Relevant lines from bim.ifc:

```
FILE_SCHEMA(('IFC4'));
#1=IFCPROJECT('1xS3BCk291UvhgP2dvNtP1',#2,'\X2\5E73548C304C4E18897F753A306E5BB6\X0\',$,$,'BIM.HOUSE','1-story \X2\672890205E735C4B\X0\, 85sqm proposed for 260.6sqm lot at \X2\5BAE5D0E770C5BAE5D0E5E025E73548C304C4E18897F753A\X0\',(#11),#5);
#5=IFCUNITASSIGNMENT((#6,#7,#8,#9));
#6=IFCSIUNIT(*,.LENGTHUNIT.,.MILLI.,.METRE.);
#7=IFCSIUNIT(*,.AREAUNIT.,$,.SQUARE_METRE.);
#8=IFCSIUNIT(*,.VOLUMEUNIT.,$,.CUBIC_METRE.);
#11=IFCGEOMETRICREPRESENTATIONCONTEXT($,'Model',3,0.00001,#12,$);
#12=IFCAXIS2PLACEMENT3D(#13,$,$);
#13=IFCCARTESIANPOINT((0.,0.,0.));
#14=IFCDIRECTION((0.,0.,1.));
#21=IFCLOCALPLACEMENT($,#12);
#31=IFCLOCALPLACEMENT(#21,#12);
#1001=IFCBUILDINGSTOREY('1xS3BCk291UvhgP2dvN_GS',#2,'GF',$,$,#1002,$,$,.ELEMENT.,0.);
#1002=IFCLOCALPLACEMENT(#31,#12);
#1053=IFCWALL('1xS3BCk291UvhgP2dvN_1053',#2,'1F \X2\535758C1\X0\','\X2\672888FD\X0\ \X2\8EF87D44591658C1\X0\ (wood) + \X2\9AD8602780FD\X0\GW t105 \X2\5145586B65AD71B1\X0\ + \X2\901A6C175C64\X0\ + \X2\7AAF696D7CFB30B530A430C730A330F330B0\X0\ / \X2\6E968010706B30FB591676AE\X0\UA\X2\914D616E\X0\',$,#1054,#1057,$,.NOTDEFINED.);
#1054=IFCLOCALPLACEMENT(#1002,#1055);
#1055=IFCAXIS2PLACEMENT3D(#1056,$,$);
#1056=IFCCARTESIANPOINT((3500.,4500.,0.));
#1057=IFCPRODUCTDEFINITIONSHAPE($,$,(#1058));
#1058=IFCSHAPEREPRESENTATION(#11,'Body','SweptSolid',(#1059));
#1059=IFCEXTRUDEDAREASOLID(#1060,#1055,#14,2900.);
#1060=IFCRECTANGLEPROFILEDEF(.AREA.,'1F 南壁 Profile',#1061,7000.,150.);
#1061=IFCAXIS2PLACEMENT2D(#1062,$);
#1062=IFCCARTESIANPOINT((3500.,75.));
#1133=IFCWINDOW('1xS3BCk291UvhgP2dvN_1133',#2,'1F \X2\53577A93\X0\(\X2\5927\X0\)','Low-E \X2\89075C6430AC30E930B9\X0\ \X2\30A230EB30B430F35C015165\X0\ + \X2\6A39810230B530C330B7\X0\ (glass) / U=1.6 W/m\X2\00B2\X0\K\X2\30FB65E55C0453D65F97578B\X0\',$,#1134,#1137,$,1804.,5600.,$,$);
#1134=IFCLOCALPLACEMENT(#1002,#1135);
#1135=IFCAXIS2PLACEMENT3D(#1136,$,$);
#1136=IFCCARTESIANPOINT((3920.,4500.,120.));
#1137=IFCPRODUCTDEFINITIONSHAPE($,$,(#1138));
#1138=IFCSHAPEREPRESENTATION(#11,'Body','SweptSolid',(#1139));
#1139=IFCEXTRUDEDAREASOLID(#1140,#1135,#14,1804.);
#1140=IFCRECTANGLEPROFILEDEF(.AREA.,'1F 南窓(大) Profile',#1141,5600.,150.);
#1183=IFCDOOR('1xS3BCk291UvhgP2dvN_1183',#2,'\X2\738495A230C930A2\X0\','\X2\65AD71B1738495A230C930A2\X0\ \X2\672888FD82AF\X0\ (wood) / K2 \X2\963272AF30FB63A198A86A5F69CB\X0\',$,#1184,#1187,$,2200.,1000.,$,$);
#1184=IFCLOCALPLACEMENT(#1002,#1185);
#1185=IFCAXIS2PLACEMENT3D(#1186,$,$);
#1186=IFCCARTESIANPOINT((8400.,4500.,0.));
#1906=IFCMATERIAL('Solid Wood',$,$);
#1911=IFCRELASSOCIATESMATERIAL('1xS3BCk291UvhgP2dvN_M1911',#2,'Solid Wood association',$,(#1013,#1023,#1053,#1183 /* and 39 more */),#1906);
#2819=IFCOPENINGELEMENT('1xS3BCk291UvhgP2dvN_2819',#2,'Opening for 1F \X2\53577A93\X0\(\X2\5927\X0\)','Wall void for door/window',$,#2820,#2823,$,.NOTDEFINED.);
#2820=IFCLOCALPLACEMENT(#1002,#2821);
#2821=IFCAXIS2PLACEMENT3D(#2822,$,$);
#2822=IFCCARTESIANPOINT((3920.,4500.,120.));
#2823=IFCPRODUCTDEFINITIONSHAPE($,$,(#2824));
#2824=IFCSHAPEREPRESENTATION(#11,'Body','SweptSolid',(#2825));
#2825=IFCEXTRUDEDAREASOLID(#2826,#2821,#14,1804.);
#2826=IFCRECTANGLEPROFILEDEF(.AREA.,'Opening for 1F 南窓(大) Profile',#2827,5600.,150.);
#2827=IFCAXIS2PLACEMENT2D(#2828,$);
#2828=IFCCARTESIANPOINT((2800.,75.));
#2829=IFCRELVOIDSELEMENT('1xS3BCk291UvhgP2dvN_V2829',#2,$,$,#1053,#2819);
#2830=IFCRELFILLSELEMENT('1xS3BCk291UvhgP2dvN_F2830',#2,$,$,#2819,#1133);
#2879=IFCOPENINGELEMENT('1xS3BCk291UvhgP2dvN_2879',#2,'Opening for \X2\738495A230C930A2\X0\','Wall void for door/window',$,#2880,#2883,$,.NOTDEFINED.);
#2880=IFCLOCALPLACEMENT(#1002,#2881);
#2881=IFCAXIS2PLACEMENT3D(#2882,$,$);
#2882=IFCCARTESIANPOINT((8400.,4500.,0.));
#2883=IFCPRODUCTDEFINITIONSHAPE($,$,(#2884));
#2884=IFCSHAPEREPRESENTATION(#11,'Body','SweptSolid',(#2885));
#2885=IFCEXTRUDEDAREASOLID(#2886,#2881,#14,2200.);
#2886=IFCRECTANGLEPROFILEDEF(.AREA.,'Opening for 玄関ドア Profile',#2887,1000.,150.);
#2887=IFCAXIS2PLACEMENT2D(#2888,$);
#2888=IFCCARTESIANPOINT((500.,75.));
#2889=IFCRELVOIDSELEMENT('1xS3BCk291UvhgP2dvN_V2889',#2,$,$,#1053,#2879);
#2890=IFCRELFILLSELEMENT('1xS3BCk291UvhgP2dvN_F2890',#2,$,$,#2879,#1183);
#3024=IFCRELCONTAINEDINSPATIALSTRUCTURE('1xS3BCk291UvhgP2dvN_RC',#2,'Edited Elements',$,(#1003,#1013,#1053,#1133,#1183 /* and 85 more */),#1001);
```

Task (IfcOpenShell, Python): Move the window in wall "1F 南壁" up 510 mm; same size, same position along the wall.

```python
import numpy as np
import ifcopenshell
import ifcopenshell.api.geometry
import ifcopenshell.util.placement
import ifcopenshell.util.unit

model = ifcopenshell.open("bim.ifc")
unit_scale = ifcopenshell.util.unit.calculate_unit_scale(model)

window = model.by_guid("1xS3BCk291UvhgP2dvN_1133")
opening = window.FillsVoids[0].RelatingOpeningElement
dz = 0.51 / unit_scale

shift = np.array([0.0, 0.0, dz])
# The window is not placed relative to its opening, so move both.
for product in (opening, window):
    matrix = ifcopenshell.util.placement.get_local_placement(product.ObjectPlacement)
    matrix[:3, 3] += shift
    ifcopenshell.api.geometry.edit_object_placement(model, product=product, matrix=matrix, is_si=False)

print(f"moved by {dz * unit_scale:+.3f} m")

model.write("bim_edited.ifc")
```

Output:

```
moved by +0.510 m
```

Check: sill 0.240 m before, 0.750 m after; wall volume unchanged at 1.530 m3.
